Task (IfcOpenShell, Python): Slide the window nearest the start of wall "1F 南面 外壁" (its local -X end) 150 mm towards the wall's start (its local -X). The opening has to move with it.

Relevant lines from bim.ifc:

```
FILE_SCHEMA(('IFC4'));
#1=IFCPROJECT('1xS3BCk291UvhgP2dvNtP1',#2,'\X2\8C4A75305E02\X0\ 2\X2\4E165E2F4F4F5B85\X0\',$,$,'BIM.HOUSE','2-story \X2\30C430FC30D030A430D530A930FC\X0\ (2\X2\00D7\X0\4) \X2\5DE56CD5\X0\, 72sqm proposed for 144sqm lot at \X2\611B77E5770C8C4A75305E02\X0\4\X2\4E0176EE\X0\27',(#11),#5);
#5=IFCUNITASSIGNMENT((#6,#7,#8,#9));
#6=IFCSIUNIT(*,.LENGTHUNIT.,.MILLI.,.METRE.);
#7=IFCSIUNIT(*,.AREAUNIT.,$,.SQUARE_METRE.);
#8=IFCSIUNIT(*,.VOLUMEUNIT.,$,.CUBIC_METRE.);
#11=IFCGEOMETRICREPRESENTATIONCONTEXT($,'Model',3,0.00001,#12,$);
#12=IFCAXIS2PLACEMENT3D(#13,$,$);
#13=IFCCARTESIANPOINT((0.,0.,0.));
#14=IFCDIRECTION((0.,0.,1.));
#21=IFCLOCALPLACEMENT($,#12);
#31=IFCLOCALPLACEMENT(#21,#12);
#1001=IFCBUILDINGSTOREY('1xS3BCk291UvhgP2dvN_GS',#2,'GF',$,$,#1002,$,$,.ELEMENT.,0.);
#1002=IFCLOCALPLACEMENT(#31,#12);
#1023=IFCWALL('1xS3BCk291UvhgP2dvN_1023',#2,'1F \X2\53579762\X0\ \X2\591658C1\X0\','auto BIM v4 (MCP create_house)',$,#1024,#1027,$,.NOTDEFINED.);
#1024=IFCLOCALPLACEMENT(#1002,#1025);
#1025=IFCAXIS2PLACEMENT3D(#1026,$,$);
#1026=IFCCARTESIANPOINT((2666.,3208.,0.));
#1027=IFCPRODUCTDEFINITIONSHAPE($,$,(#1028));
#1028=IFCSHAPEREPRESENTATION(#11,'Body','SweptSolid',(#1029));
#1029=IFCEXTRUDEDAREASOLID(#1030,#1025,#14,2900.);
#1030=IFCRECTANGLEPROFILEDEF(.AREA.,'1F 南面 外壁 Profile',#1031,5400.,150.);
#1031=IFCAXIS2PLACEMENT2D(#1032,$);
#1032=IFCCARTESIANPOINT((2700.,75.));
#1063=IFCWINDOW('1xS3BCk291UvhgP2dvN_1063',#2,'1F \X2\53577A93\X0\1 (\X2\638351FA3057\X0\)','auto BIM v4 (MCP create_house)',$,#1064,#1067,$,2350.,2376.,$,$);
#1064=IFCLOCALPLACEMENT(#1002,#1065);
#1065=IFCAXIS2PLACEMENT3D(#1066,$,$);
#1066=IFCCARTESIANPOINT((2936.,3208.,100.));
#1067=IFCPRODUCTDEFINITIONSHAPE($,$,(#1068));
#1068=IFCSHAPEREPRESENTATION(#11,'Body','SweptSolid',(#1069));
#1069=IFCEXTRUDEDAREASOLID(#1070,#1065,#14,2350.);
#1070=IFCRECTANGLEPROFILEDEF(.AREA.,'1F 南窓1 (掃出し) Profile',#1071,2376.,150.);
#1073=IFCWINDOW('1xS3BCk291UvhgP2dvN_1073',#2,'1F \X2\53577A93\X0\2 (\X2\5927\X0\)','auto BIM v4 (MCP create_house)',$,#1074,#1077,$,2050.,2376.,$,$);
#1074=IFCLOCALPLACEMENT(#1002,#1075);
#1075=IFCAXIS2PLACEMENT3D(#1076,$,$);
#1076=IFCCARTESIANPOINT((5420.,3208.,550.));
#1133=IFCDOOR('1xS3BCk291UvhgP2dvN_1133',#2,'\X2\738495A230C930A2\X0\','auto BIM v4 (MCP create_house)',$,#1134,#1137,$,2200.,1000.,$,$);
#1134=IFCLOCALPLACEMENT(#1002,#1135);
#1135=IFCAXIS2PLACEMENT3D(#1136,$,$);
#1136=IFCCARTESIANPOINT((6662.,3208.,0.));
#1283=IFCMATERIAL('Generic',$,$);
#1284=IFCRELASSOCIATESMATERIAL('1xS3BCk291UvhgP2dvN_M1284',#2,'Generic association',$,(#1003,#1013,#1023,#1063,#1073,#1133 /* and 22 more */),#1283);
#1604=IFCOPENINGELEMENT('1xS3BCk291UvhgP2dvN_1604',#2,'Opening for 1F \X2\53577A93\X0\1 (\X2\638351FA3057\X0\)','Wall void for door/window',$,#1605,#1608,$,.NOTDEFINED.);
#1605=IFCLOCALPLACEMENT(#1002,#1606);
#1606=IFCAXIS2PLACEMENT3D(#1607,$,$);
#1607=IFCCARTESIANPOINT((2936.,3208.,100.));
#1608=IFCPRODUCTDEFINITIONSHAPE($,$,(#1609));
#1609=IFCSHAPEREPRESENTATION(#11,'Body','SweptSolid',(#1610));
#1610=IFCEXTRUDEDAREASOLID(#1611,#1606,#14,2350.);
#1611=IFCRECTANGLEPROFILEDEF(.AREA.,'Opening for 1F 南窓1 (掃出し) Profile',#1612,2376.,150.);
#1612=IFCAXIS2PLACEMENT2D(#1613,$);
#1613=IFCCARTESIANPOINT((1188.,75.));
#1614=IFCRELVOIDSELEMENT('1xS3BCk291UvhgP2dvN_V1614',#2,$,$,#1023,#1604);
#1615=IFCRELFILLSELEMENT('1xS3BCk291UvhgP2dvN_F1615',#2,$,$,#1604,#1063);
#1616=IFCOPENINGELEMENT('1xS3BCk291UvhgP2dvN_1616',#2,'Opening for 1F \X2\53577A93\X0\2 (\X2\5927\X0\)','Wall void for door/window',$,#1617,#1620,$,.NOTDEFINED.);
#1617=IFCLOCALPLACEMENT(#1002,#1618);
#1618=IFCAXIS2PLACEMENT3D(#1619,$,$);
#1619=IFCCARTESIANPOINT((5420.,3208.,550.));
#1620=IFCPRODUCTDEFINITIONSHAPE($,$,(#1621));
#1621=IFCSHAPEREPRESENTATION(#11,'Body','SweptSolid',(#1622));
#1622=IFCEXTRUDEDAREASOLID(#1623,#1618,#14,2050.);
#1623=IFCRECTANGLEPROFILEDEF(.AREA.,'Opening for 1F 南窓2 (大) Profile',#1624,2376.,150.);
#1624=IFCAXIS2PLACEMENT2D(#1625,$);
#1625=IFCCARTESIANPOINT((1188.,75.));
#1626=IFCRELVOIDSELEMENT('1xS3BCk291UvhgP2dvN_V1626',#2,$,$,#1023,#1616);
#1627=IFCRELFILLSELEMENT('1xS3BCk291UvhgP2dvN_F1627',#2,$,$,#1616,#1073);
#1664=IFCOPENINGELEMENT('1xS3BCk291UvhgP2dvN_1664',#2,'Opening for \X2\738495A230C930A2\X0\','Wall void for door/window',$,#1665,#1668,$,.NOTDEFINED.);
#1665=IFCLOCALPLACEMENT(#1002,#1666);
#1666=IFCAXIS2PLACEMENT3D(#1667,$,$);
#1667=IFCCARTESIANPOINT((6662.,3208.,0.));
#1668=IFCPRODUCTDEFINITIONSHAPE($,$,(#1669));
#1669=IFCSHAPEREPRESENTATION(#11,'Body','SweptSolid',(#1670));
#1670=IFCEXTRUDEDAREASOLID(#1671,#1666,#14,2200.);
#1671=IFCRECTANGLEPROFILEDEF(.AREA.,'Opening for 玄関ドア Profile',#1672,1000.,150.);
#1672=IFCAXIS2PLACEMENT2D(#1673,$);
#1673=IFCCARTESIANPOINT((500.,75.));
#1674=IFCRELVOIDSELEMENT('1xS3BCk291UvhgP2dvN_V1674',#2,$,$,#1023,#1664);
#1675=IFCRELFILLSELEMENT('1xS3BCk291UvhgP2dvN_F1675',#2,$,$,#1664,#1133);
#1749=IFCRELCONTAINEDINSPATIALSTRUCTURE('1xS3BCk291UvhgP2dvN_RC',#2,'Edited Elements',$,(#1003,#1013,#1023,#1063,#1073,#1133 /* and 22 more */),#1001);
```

```python
import ifcopenshell
import ifcopenshell.api.geometry
import ifcopenshell.util.placement
import ifcopenshell.util.unit

model = ifcopenshell.open("bim.ifc")
unit_scale = ifcopenshell.util.unit.calculate_unit_scale(model)

window = model.by_id(1063)
opening = window.FillsVoids[0].RelatingOpeningElement
wall = opening.VoidsElements[0].RelatingBuildingElement

wall_matrix = ifcopenshell.util.placement.get_local_placement(wall.ObjectPlacement)
shift = wall_matrix[:3, 0] * -0.15 / unit_scale
before = ifcopenshell.util.placement.get_local_placement(window.ObjectPlacement)[:3, 3].copy()

# The window is not placed relative to its opening, so move both.
for product in (opening, window):
    matrix = ifcopenshell.util.placement.get_local_placement(product.ObjectPlacement)
    matrix[:3, 3] += shift
    ifcopenshell.api.geometry.edit_object_placement(model, product=product, matrix=matrix, is_si=False)

after = ifcopenshell.util.placement.get_local_placement(window.ObjectPlacement)[:3, 3]
print("window moved by", (after - before).round(3) + 0.0)

model.write("bim_v2.ifc")
```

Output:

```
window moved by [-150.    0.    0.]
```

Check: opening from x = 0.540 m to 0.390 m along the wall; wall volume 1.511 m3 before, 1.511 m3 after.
